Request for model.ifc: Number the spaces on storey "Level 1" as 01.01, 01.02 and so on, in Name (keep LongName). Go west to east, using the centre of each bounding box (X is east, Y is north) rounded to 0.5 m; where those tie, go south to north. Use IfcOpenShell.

First a look at what the model holds.

```python
import ifcopenshell
import ifcopenshell.util.element
import ifcopenshell.util.placement

model = ifcopenshell.open("model.ifc")
print(model.schema)
storey = next(s for s in model.by_type("IfcBuildingStorey") if s.Name == "Level 1")
spaces = [e for e in ifcopenshell.util.element.get_decomposition(storey) if e.is_a("IfcSpace")]
for e in sorted(spaces, key=lambda e: e.id()):
    origin = ifcopenshell.util.placement.get_local_placement(e.ObjectPlacement)[:3, 3]
    print(e.id(), e.Name, e.LongName, origin.round(2) + 0.0, sep=" | ")
```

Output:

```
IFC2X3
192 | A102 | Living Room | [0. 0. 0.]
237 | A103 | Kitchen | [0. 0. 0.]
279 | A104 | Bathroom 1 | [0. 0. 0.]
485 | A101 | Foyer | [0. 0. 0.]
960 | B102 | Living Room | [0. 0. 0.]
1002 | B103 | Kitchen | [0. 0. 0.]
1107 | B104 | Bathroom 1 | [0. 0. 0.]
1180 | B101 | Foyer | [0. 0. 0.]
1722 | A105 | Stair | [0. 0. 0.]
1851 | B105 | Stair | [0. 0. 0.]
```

```python
import ifcopenshell
import ifcopenshell.geom
import ifcopenshell.util.element
import ifcopenshell.util.shape

model = ifcopenshell.open("model.ifc")
settings = ifcopenshell.geom.settings()
settings.set("use-world-coords", True)


def centre(element):
    shape = ifcopenshell.geom.create_shape(settings, element)
    return ifcopenshell.util.shape.get_bbox_centroid(shape.geometry)


storey = next(s for s in model.by_type("IfcBuildingStorey") if s.Name == "Level 1")
spaces = [e for e in ifcopenshell.util.element.get_decomposition(storey) if e.is_a("IfcSpace")]

# Insertion points can sit at a corner or the storey origin, so sort by the geometry (in metres).
centres = {e: centre(e) for e in spaces}
spaces.sort(key=lambda e: (round(centres[e][0] / 0.5), centres[e][1]))

for i, e in enumerate(spaces, start=1):
    number = f"01.{i:02d}"
    e.Name = number
    print(e.id(), number)

model.write("model-out.ifc")
```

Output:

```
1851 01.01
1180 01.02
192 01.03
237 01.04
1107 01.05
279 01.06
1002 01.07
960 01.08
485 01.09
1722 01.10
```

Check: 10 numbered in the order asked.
